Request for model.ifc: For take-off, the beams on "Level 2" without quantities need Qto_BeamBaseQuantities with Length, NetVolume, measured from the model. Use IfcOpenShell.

First a look at what the model holds.

```python
import ifcopenshell
import ifcopenshell.util.element
import ifcopenshell.util.unit

model = ifcopenshell.open("model.ifc")
print(model.schema)
for unit_type in ("LENGTHUNIT", "AREAUNIT", "VOLUMEUNIT"):
    print(unit_type, ifcopenshell.util.unit.calculate_unit_scale(model, unit_type))
storey = next(s for s in model.by_type("IfcBuildingStorey") if s.Name == "Level 2")
beams = [e for e in ifcopenshell.util.element.get_decomposition(storey) if e.is_a("IfcBeam")]
for e in sorted(beams, key=lambda e: e.id()):
    print(e.id(), e.is_a(), e.Name, list(ifcopenshell.util.element.get_psets(e, qtos_only=True)), sep=" | ")
```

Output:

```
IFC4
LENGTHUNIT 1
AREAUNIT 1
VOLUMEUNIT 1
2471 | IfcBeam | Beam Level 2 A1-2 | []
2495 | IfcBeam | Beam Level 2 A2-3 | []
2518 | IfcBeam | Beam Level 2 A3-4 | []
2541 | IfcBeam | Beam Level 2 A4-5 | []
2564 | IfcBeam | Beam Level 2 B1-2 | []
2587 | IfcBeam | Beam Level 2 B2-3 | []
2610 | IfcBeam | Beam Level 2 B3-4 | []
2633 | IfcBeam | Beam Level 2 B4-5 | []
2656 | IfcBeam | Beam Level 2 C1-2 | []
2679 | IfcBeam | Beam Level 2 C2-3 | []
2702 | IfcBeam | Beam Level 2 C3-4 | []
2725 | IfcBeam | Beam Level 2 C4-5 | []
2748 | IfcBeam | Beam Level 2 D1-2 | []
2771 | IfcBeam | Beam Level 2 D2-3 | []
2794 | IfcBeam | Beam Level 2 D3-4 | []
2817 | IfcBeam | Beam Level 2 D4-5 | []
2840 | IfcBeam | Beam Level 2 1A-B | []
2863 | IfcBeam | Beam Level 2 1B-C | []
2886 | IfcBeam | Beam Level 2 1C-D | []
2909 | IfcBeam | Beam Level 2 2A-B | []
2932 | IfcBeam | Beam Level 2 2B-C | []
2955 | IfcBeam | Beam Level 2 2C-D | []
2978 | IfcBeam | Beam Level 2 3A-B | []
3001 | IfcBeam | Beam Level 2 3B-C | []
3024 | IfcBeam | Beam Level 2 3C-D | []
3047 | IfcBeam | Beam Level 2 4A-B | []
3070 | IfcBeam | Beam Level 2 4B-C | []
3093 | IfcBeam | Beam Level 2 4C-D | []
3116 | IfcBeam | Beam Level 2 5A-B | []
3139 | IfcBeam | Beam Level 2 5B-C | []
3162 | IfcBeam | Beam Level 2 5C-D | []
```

```python
import ifcopenshell
import ifcopenshell.api.pset
import ifcopenshell.geom
import ifcopenshell.util.element
import ifcopenshell.util.shape
import ifcopenshell.util.unit

model = ifcopenshell.open("model.ifc")
unit_scale = ifcopenshell.util.unit.calculate_unit_scale(model)
volume_scale = ifcopenshell.util.unit.calculate_unit_scale(model, "VOLUMEUNIT")
settings = ifcopenshell.geom.settings()

storey = next(s for s in model.by_type("IfcBuildingStorey") if s.Name == "Level 2")
beams = [e for e in ifcopenshell.util.element.get_decomposition(storey) if e.is_a("IfcBeam")]

for e in sorted(beams, key=lambda e: e.id()):
    if ifcopenshell.util.element.get_psets(e, qtos_only=True, should_inherit=False):
        continue
    # Geometry comes back in metres, in the element's own axes.
    shape = ifcopenshell.geom.create_shape(settings, e)
    values = {
        "Length": ifcopenshell.util.shape.get_max_xyz(shape.geometry) / unit_scale,
        "NetVolume": ifcopenshell.util.shape.get_volume(shape.geometry) / volume_scale,
    }
    qto = ifcopenshell.api.pset.add_qto(model, product=e, name="Qto_BeamBaseQuantities")
    ifcopenshell.api.pset.edit_qto(model, qto=qto, properties=values)
    print(e.id(), {k: round(v, 3) for k, v in values.items()})

model.write("model_v2.ifc")
```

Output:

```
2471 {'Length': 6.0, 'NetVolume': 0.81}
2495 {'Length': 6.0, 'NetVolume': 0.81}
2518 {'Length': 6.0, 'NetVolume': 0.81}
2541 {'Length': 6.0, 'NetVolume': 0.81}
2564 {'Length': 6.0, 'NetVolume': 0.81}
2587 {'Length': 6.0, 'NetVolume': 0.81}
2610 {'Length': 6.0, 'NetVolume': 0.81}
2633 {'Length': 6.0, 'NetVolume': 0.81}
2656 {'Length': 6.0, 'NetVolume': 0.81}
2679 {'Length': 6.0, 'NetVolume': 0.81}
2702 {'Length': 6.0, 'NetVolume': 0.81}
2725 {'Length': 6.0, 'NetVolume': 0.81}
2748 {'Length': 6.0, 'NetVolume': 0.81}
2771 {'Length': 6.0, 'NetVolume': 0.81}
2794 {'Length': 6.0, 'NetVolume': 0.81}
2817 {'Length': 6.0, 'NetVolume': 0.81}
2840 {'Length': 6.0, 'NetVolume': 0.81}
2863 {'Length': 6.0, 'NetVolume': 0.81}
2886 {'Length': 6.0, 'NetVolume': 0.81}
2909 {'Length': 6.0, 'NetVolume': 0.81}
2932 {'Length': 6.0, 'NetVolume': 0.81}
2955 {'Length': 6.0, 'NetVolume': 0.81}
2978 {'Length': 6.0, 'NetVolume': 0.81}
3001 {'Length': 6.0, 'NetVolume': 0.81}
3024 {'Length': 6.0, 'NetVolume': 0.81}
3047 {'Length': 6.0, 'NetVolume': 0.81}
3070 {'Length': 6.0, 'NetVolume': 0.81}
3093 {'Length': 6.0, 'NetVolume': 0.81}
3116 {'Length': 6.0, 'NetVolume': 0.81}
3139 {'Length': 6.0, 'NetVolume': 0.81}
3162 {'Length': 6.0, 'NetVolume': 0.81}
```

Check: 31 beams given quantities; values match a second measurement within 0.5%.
